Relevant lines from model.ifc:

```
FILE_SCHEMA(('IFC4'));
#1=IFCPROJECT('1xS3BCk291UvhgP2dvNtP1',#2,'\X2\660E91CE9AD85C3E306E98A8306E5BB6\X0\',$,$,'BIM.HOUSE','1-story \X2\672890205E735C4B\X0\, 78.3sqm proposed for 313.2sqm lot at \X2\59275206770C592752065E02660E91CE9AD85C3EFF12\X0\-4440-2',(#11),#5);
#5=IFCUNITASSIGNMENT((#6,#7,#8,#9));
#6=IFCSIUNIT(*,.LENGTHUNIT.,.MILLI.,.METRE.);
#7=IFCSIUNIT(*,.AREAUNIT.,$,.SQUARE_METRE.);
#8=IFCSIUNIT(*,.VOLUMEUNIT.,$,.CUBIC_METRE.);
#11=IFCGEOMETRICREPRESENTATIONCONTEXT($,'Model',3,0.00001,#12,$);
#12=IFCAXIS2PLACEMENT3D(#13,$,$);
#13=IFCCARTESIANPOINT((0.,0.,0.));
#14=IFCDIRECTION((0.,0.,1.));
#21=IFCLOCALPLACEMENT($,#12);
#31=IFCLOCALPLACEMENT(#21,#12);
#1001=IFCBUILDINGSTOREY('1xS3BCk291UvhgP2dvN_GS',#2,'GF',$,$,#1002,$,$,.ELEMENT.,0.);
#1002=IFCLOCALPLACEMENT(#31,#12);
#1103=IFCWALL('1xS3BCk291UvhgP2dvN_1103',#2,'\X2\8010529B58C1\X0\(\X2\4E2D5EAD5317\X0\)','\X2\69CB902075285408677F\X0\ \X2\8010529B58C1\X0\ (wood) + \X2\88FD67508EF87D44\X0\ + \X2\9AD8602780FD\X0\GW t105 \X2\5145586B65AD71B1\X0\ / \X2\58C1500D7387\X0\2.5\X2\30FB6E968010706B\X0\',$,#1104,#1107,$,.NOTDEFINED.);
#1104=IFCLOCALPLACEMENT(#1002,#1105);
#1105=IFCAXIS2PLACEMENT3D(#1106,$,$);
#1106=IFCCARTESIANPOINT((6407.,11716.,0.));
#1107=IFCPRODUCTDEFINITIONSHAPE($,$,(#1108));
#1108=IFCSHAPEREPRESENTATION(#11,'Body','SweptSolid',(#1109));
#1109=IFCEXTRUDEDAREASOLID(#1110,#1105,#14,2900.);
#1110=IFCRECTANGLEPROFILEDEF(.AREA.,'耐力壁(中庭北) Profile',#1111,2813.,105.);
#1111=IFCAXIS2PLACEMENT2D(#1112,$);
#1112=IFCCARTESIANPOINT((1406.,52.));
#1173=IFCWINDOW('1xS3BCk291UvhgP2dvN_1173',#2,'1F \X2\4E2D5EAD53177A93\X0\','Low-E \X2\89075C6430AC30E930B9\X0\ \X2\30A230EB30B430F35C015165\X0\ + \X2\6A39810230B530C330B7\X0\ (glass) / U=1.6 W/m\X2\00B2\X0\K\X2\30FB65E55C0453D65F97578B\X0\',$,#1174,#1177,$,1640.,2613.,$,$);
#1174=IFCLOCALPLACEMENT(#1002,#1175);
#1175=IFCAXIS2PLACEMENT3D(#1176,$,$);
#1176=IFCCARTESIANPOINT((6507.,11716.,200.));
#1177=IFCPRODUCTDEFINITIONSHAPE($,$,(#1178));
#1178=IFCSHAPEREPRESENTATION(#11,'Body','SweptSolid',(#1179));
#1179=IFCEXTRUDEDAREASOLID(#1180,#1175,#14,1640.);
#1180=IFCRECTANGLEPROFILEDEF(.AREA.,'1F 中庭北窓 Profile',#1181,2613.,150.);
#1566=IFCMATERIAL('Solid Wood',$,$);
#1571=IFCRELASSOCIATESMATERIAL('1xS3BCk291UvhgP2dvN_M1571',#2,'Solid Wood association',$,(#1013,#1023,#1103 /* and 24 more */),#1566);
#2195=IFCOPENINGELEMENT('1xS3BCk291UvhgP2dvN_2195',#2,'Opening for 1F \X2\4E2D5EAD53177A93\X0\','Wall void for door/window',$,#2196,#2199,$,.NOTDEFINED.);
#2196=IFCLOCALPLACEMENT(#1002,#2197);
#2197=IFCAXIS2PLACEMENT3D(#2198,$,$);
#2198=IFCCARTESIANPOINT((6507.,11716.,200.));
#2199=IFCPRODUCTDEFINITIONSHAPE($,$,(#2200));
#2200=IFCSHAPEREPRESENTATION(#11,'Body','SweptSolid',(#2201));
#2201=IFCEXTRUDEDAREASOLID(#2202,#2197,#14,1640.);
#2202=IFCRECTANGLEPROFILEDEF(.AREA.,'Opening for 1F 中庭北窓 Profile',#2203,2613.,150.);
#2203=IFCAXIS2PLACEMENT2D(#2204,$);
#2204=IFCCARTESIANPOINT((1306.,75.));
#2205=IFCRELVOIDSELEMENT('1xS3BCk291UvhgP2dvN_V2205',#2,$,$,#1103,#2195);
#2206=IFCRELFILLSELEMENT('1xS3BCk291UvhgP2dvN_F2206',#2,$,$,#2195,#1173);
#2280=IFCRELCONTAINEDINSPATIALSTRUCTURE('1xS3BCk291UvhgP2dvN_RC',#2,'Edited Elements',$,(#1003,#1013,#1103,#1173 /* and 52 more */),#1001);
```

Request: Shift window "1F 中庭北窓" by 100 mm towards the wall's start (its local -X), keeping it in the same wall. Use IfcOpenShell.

```python
import ifcopenshell
import ifcopenshell.api.geometry
import ifcopenshell.util.placement

model = ifcopenshell.open("model.ifc")

window = model.by_guid("1xS3BCk291UvhgP2dvN_1173")
opening = window.FillsVoids[0].RelatingOpeningElement
wall = opening.VoidsElements[0].RelatingBuildingElement

wall_matrix = ifcopenshell.util.placement.get_local_placement(wall.ObjectPlacement)
shift = wall_matrix[:3, 0] * -100.0
before = ifcopenshell.util.placement.get_local_placement(window.ObjectPlacement)[:3, 3].copy()

# The window is not placed relative to its opening, so move both.
for product in (opening, window):
    matrix = ifcopenshell.util.placement.get_local_placement(product.ObjectPlacement)
    matrix[:3, 3] += shift
    ifcopenshell.api.geometry.edit_object_placement(model, product=product, matrix=matrix, is_si=False)

after = ifcopenshell.util.placement.get_local_placement(window.ObjectPlacement)[:3, 3]
print("window moved by", (after - before).round(3) + 0.0)

model.write("model_updated.ifc")
```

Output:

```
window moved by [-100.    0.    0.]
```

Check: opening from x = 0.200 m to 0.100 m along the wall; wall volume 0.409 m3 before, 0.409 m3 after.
